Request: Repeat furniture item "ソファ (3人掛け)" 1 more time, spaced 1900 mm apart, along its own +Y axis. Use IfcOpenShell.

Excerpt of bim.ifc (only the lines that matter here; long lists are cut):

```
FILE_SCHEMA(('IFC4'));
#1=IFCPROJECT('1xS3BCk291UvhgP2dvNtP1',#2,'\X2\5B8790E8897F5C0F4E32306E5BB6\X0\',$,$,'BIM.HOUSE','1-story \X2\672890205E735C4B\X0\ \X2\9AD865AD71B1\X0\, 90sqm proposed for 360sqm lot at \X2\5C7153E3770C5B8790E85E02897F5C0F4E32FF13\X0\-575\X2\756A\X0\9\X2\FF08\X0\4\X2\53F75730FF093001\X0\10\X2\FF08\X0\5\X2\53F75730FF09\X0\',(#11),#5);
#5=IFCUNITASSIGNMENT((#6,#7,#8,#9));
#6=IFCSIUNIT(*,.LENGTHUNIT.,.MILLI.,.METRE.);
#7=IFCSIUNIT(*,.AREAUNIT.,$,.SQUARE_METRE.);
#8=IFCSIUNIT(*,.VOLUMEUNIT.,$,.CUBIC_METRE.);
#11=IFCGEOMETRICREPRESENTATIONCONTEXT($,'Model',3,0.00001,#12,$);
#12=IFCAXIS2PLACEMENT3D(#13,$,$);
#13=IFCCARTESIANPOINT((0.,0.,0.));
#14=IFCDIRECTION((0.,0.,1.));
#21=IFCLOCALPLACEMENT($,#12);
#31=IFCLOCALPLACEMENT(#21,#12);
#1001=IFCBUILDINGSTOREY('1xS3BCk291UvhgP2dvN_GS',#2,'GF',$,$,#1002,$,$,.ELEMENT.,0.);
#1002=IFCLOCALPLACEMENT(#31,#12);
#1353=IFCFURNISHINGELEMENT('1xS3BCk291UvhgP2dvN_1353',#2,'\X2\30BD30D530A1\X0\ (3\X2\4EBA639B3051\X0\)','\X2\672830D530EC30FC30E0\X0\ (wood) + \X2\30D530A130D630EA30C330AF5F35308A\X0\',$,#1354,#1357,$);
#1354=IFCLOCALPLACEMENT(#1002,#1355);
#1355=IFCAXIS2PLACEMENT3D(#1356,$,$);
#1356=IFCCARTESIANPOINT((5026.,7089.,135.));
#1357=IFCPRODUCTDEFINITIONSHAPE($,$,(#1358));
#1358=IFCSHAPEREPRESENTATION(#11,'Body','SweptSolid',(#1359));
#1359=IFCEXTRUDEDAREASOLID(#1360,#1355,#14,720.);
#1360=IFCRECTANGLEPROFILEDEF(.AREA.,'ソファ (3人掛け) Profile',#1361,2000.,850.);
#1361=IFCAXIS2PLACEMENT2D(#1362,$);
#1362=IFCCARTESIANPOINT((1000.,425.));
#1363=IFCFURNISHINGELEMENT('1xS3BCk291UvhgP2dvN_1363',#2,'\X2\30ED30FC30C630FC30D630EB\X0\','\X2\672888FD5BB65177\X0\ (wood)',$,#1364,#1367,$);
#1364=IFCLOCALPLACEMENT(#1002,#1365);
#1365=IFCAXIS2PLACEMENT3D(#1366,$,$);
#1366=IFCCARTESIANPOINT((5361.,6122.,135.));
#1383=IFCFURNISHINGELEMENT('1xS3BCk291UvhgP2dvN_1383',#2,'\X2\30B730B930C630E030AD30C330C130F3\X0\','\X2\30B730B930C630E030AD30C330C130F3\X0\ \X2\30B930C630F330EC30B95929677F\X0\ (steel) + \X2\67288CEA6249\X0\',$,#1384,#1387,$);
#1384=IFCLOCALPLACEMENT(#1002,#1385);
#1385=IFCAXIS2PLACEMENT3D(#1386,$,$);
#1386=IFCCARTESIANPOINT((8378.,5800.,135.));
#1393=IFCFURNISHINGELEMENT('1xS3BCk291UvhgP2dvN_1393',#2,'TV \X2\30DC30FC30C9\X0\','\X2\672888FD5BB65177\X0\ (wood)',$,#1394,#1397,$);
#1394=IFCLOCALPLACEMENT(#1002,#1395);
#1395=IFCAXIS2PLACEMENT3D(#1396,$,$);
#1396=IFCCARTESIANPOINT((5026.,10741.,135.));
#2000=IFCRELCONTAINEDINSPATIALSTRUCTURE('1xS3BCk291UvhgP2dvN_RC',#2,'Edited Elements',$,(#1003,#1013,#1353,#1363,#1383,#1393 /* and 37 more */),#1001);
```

```python
import ifcopenshell
import ifcopenshell.api.geometry
import ifcopenshell.api.root
import ifcopenshell.util.element
import ifcopenshell.util.placement

model = ifcopenshell.open("bim.ifc")


def reuse_history(source, copy):
    """copy_class also copies each property set's owner history, people and application; keep the originals."""
    for rel in copy.IsDefinedBy:
        if rel.is_a("IfcRelDefinesByProperties") and (history := rel.RelatingPropertyDefinition.OwnerHistory):
            rel.RelatingPropertyDefinition.OwnerHistory = source.OwnerHistory
            ifcopenshell.util.element.remove_deep2(model, history)


source = model.by_guid("1xS3BCk291UvhgP2dvN_1353")
base = ifcopenshell.util.placement.get_local_placement(source.ObjectPlacement)
step = base[:3, 1] * 1900.0

for i in range(1, 2):
    copy = ifcopenshell.api.root.copy_class(model, product=source)
    copy.Representation = ifcopenshell.util.element.copy_deep(
        model, source.Representation, exclude=["IfcGeometricRepresentationContext", "IfcRepresentationMap"]
    )
    reuse_history(source, copy)
    matrix = base.copy()
    matrix[:3, 3] += i * step
    print("added at", matrix[:3, 3].round(3) + 0.0)
    ifcopenshell.api.geometry.edit_object_placement(model, product=copy, matrix=matrix, is_si=False)

model.write("bim_edited.ifc")
```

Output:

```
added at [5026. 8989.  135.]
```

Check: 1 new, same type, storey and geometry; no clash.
